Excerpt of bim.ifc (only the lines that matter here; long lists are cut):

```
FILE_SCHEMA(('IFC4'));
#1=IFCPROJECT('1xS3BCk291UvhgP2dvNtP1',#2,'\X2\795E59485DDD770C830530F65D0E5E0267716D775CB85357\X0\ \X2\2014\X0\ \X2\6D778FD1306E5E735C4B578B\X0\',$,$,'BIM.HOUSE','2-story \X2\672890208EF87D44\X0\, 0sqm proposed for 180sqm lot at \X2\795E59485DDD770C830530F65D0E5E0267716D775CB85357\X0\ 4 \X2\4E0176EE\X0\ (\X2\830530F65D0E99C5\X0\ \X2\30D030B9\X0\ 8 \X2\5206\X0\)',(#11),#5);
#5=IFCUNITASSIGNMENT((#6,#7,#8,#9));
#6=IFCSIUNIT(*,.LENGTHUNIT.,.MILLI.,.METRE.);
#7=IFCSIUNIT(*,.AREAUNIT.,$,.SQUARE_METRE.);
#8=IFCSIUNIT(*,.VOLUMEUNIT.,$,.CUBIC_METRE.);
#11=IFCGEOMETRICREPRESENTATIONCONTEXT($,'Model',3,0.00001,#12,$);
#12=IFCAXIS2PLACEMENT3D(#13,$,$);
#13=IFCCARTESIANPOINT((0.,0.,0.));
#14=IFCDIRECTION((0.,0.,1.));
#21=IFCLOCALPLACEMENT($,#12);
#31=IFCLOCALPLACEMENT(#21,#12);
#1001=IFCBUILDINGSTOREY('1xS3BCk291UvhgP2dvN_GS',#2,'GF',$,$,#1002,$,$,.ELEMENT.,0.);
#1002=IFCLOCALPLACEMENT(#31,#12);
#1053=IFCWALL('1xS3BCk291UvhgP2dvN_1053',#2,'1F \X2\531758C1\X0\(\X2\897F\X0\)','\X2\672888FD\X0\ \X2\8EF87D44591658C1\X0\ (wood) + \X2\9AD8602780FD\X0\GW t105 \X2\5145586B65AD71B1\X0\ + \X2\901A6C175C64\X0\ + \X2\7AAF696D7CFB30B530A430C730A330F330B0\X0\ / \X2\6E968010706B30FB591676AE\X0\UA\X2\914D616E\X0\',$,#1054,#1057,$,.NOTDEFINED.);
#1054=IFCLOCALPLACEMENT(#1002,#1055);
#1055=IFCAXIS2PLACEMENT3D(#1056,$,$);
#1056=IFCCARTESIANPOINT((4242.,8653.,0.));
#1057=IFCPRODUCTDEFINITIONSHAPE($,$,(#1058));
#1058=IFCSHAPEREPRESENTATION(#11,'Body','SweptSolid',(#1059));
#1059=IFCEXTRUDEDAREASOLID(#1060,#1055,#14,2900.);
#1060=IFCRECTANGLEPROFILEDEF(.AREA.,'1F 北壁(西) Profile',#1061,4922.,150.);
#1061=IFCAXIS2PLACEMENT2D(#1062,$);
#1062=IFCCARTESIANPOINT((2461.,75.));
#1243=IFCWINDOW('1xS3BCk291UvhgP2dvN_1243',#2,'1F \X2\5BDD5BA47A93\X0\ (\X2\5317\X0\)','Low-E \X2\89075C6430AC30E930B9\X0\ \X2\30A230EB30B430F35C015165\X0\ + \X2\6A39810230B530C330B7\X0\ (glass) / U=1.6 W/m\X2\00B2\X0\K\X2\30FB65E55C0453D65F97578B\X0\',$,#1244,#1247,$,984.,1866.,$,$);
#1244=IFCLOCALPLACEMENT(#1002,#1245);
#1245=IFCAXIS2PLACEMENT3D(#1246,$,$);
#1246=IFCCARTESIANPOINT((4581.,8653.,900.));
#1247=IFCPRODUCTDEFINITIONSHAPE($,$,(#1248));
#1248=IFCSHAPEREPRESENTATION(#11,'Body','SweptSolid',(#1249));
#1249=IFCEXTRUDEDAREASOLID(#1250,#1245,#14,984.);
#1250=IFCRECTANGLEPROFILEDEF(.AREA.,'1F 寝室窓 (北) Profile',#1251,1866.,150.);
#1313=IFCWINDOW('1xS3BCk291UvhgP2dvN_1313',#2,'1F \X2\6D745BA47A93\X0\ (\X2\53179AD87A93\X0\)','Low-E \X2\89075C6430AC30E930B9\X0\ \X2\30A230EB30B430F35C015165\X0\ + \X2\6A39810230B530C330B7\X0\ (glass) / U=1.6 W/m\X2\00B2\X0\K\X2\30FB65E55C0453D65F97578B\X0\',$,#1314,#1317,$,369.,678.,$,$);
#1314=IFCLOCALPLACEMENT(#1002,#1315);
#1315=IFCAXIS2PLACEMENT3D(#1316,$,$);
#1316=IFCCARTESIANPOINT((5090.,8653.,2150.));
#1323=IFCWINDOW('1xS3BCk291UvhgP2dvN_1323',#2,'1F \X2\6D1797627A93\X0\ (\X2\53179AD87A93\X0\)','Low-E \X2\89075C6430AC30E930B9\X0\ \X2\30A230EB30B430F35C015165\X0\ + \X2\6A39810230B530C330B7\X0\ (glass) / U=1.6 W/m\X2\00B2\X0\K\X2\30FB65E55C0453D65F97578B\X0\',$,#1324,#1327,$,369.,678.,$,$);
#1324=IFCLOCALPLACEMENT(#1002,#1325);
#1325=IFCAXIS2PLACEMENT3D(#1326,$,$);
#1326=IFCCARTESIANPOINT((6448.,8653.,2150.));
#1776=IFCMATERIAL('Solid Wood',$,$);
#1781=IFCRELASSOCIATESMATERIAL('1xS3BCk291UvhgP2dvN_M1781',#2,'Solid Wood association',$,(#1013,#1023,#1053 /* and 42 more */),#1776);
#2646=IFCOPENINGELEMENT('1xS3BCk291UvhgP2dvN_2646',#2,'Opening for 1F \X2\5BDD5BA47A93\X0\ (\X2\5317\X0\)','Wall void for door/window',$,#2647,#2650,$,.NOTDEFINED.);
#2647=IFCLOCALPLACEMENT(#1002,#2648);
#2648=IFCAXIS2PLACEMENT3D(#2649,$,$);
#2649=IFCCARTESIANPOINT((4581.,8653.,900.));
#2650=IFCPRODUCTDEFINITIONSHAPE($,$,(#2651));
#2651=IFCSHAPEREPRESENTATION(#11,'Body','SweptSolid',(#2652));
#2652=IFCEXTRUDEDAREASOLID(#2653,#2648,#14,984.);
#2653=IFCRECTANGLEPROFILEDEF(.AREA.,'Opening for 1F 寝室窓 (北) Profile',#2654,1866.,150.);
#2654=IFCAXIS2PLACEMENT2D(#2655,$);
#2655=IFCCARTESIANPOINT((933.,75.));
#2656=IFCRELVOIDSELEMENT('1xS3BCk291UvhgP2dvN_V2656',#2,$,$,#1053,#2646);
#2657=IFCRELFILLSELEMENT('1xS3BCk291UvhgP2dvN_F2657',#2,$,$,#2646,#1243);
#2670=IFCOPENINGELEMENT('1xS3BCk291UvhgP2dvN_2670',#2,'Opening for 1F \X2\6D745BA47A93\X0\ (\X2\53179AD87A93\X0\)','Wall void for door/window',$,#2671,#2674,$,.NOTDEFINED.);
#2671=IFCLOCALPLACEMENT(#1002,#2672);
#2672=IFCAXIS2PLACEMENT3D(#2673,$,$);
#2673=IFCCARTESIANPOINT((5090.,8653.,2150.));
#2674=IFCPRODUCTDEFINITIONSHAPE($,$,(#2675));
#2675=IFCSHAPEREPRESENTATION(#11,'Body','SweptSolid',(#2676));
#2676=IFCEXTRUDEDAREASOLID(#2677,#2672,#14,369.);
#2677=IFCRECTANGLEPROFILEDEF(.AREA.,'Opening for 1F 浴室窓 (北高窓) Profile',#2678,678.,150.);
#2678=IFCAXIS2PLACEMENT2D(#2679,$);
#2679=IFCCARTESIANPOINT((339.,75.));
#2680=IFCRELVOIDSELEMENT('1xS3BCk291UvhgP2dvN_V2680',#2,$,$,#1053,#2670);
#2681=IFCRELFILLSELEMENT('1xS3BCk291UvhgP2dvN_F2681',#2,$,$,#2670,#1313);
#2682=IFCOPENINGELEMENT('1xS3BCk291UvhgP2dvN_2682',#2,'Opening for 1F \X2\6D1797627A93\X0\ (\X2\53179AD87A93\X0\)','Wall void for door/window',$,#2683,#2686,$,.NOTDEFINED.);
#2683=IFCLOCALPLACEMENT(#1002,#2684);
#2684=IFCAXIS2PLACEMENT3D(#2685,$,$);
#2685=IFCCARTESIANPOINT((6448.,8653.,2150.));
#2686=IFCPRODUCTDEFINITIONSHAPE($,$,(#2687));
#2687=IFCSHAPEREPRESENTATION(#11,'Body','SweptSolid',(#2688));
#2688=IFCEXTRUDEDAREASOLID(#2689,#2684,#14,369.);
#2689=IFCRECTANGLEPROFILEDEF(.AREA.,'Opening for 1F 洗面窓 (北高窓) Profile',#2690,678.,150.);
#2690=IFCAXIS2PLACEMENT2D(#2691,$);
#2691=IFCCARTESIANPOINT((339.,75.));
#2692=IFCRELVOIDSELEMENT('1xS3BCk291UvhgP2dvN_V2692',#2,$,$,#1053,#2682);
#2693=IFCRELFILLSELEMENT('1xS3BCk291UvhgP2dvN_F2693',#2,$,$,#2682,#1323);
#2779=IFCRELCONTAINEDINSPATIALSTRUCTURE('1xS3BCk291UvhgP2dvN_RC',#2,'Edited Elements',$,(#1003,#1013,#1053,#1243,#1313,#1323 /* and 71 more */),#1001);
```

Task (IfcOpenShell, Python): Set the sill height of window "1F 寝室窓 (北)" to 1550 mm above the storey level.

```python
import numpy as np
import ifcopenshell
import ifcopenshell.api.geometry
import ifcopenshell.geom
import ifcopenshell.util.element
import ifcopenshell.util.placement
import ifcopenshell.util.shape
import ifcopenshell.util.unit

model = ifcopenshell.open("bim.ifc")
unit_scale = ifcopenshell.util.unit.calculate_unit_scale(model)

window = model.by_id(1243)
opening = window.FillsVoids[0].RelatingOpeningElement
storey = ifcopenshell.util.element.get_container(window, ifc_class="IfcBuildingStorey")
level = ifcopenshell.util.placement.get_local_placement(storey.ObjectPlacement)[2, 3]

# The opening's origin need not be at the sill, so measure its lowest point.
shape = ifcopenshell.geom.create_shape(ifcopenshell.geom.settings(), opening)
bottom = ifcopenshell.util.shape.get_shape_bottom_elevation(shape, shape.geometry) / unit_scale
dz = level + 1550.0 - bottom

shift = np.array([0.0, 0.0, dz])
# The window is not placed relative to its opening, so move both.
for product in (opening, window):
    matrix = ifcopenshell.util.placement.get_local_placement(product.ObjectPlacement)
    matrix[:3, 3] += shift
    ifcopenshell.api.geometry.edit_object_placement(model, product=product, matrix=matrix, is_si=False)

print(f"moved by {dz * unit_scale:+.3f} m")

model.write("bim_updated.ifc")
```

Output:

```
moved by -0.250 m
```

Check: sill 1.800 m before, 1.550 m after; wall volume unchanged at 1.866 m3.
